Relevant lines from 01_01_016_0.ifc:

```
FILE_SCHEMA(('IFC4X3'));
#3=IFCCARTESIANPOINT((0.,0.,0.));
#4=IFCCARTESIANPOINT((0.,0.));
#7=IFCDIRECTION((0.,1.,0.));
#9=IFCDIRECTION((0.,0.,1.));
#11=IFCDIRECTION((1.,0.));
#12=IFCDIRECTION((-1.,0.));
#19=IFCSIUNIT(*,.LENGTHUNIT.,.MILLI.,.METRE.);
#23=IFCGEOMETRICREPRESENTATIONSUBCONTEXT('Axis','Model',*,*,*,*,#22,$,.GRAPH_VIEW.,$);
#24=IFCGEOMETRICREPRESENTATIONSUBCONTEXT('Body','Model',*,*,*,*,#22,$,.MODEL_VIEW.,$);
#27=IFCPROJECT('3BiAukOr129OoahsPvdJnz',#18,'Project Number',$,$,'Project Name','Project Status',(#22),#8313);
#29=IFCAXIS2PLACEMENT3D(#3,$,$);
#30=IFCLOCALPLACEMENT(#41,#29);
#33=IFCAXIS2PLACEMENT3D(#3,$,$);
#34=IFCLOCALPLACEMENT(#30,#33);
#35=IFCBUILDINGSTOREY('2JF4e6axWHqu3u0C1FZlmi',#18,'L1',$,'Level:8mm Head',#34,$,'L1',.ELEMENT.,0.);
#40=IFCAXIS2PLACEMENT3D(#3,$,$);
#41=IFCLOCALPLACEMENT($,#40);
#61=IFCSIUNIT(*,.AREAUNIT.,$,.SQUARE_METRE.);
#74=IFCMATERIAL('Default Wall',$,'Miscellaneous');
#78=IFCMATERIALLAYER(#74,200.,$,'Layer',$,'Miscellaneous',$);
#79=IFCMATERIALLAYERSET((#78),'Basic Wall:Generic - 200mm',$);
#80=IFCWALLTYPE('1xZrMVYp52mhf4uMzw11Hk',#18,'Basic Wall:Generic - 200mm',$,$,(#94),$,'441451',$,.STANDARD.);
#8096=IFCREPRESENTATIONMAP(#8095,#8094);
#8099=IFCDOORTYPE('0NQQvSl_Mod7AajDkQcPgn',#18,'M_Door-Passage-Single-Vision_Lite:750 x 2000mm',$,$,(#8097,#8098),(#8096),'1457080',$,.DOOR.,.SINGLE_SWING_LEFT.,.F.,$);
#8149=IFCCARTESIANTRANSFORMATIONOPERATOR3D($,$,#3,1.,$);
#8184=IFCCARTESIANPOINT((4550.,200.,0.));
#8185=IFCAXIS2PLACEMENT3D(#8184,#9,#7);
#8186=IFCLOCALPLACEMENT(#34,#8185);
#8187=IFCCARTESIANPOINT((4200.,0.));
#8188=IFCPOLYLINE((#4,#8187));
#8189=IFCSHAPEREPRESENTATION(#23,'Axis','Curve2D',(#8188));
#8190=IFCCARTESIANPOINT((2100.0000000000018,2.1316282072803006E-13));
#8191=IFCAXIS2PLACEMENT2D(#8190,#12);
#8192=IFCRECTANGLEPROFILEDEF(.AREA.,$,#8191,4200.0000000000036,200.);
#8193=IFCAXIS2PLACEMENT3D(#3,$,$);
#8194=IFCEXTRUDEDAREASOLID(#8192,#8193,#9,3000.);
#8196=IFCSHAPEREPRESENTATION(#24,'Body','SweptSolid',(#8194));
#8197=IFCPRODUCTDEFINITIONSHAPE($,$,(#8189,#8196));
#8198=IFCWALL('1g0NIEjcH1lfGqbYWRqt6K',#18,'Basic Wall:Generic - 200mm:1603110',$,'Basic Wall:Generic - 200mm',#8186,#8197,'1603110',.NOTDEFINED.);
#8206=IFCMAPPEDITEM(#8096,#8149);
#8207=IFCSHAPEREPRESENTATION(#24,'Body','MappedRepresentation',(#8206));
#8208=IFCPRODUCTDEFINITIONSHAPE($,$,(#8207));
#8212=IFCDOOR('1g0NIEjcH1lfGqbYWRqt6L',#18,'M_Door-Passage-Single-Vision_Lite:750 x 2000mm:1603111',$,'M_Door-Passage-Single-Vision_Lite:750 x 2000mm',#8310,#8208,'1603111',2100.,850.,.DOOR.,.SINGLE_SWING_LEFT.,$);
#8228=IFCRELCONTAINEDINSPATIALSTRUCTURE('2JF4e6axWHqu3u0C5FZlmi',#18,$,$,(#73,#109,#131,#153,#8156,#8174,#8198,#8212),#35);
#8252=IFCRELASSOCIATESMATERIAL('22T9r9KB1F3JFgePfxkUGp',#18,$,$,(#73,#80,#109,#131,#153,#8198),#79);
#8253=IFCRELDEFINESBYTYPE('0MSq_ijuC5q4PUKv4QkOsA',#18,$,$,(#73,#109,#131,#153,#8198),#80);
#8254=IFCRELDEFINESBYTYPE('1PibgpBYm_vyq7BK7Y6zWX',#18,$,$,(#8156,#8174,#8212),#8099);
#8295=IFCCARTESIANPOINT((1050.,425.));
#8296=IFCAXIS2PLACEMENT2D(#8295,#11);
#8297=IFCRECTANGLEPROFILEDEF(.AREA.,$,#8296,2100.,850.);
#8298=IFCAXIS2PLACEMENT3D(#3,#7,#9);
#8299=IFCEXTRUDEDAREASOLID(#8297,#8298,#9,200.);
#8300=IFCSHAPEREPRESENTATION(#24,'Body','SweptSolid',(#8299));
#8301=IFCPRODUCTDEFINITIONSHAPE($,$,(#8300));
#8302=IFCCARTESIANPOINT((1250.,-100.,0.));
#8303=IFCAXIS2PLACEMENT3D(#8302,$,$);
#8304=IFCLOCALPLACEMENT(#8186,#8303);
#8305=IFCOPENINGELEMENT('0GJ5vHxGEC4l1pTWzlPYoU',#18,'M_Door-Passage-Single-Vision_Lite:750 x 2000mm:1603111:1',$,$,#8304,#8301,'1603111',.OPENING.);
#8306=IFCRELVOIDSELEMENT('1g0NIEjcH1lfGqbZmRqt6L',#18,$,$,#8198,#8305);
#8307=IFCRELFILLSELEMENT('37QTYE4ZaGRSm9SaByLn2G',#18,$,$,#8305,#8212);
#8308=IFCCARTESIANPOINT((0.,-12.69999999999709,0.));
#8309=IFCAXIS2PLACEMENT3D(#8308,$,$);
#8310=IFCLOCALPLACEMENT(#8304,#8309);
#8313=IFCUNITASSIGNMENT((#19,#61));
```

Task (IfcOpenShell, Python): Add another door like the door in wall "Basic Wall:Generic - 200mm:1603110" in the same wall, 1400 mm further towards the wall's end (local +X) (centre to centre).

```python
import ifcopenshell
import ifcopenshell.api.feature
import ifcopenshell.api.geometry
import ifcopenshell.api.root
import ifcopenshell.geom
import ifcopenshell.util.element
import ifcopenshell.util.placement
import ifcopenshell.util.shape
import ifcopenshell.util.unit

model = ifcopenshell.open("01_01_016_0.ifc")
unit_scale = ifcopenshell.util.unit.calculate_unit_scale(model)
settings = ifcopenshell.geom.settings()


def volume(element):
    """Net volume in cubic metres, openings subtracted."""
    shape = ifcopenshell.geom.create_shape(settings, element)
    return ifcopenshell.util.shape.get_volume(shape.geometry)


def reuse_history(source, copy):
    """copy_class also copies each property set's owner history, people and application; keep the originals."""
    for rel in copy.IsDefinedBy:
        if rel.is_a("IfcRelDefinesByProperties") and (history := rel.RelatingPropertyDefinition.OwnerHistory):
            rel.RelatingPropertyDefinition.OwnerHistory = source.OwnerHistory
            ifcopenshell.util.element.remove_deep2(model, history)


door = model.by_id(8212)
opening = door.FillsVoids[0].RelatingOpeningElement
wall = opening.VoidsElements[0].RelatingBuildingElement
before = volume(wall)
shift = ifcopenshell.util.placement.get_local_placement(wall.ObjectPlacement)[:3, 0] * 1.4 / unit_scale

# copy_class copies the void relationship, type, container and properties, but no geometry.
new_opening = ifcopenshell.api.root.copy_class(model, product=opening)
new_opening.Representation = ifcopenshell.util.element.copy_deep(
    model, opening.Representation, exclude=["IfcGeometricRepresentationContext", "IfcRepresentationMap"]
)
new_opening.Name = "M_Door-Passage-Single-Vision_Lite:750 x 2000mm"
new_opening.Tag = None
new_door = ifcopenshell.api.root.copy_class(model, product=door)
new_door.Representation = ifcopenshell.util.element.copy_deep(
    model, door.Representation, exclude=["IfcGeometricRepresentationContext", "IfcRepresentationMap"]
)
new_door.Name = "M_Door-Passage-Single-Vision_Lite:750 x 2000mm"
new_door.Tag = None
reuse_history(door, new_door)
ifcopenshell.api.feature.add_filling(model, opening=new_opening, element=new_door)

for old, new in ((opening, new_opening), (door, new_door)):
    matrix = ifcopenshell.util.placement.get_local_placement(old.ObjectPlacement)
    matrix[:3, 3] += shift
    ifcopenshell.api.geometry.edit_object_placement(model, product=new, matrix=matrix, is_si=False)

after = volume(wall)

print(f"wall volume {before:.3f} -> {after:.3f} m3")

model.write("01_01_016_0-out.ifc")
```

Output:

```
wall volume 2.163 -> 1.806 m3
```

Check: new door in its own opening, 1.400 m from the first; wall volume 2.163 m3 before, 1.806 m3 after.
